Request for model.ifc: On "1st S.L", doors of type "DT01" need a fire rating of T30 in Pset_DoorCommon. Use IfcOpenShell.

First a look at what the model holds.

```python
import ifcopenshell
import ifcopenshell.util.element

model = ifcopenshell.open("model.ifc")
print(model.schema)
storey = next(s for s in model.by_type("IfcBuildingStorey") if s.Name == "1st S.L")
doors = [e for e in ifcopenshell.util.element.get_decomposition(storey) if e.is_a("IfcDoor")]
seen = {}
for e in doors:
    element_type = ifcopenshell.util.element.get_type(e)
    key = (element_type.Name if element_type != e and element_type else None, ifcopenshell.util.element.get_pset(e, "Pset_DoorCommon", "FireRating"))
    seen[key] = seen.get(key, 0) + 1
for (name, value), count in sorted(seen.items(), key=str):
    print(count, "x", name, "|", value)
```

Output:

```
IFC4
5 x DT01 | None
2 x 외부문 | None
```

```python
import ifcopenshell
import ifcopenshell.api.pset
import ifcopenshell.util.element

model = ifcopenshell.open("model.ifc")

storey = next(s for s in model.by_type("IfcBuildingStorey") if s.Name == "1st S.L")
doors = [e for e in ifcopenshell.util.element.get_decomposition(storey) if e.is_a("IfcDoor")]

count = 0
for e in doors:
    element_type = ifcopenshell.util.element.get_type(e)
    if element_type in (None, e) or element_type.Name != "DT01":
        continue
    # add_pset returns the element's existing set when there is one.
    pset = ifcopenshell.api.pset.add_pset(model, product=e, name="Pset_DoorCommon")
    ifcopenshell.api.pset.edit_pset(model, pset=pset, properties={"FireRating": "T30"})
    count += 1

print(count, "doors updated")

model.write("model_rev.ifc")
```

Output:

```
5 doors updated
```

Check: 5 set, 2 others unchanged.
